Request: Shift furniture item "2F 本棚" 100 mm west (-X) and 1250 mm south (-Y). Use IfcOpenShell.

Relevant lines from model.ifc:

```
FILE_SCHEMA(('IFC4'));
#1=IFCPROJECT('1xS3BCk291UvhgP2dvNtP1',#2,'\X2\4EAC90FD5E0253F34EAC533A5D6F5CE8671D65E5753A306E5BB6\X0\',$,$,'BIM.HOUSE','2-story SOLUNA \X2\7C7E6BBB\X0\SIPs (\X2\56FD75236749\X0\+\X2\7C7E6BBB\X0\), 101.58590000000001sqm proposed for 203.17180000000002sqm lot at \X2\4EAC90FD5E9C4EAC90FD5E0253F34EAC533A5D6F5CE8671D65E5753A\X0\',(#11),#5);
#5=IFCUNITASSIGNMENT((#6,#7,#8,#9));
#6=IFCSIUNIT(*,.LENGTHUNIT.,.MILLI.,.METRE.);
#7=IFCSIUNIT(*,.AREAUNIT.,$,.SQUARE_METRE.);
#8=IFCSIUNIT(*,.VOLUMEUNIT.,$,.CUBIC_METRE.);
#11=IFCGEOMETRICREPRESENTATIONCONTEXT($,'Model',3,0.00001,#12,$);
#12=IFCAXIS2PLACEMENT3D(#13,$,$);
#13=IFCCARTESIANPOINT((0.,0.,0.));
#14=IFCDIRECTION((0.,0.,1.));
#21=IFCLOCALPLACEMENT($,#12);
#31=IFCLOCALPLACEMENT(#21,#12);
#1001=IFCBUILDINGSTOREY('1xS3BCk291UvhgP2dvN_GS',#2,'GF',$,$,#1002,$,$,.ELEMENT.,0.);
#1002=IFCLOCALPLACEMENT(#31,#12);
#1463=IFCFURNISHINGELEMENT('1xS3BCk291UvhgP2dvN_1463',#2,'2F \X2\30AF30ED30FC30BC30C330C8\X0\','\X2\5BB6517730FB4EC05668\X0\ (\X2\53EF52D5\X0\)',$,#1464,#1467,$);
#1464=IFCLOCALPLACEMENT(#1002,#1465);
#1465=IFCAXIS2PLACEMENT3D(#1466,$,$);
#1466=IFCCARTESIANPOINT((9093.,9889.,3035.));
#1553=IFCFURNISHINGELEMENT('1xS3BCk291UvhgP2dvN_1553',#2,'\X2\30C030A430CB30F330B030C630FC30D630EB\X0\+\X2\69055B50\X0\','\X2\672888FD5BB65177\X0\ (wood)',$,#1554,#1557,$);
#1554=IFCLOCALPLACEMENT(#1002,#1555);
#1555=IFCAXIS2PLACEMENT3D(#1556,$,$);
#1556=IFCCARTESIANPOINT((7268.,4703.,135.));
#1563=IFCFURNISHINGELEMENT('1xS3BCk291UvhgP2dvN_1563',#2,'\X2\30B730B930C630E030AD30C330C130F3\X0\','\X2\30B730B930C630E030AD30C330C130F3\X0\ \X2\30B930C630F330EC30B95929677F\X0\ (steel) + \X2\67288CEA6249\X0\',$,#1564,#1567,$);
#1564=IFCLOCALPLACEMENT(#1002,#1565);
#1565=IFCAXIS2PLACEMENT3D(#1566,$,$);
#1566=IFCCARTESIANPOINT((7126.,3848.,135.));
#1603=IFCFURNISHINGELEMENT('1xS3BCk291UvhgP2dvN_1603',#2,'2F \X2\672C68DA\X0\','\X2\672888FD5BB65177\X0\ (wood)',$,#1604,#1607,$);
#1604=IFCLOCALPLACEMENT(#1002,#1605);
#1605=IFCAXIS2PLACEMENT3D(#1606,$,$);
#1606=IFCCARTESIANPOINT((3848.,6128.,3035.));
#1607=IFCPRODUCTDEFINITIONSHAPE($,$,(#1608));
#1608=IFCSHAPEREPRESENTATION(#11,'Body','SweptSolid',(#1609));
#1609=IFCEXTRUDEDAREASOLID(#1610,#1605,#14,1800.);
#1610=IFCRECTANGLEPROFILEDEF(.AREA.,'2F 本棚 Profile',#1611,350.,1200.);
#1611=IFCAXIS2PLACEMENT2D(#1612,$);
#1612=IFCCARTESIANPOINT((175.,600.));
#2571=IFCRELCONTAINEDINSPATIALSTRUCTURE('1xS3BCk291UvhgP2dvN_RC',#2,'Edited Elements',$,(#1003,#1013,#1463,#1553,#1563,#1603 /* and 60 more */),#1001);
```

```python
import ifcopenshell
import ifcopenshell.api.geometry
import ifcopenshell.util.placement
import ifcopenshell.util.unit

model = ifcopenshell.open("model.ifc")
unit_scale = ifcopenshell.util.unit.calculate_unit_scale(model)

item = model.by_guid("1xS3BCk291UvhgP2dvN_1603")
matrix = ifcopenshell.util.placement.get_local_placement(item.ObjectPlacement)
matrix[0, 3] -= 0.1 / unit_scale
matrix[1, 3] -= 1.25 / unit_scale
ifcopenshell.api.geometry.edit_object_placement(model, product=item, matrix=matrix, is_si=False)

print(ifcopenshell.util.placement.get_local_placement(item.ObjectPlacement).round(3) + 0.0)

model.write("model_updated.ifc")
```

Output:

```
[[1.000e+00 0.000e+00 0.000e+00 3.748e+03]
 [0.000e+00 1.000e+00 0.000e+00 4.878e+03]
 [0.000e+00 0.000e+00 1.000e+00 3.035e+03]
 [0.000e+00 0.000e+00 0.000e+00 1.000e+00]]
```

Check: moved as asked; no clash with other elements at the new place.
